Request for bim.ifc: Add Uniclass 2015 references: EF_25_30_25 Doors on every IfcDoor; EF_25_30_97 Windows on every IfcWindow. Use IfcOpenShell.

First a look at what the model holds.

```python
import ifcopenshell

model = ifcopenshell.open("bim.ifc")
print(model.schema)
print("classifications:", [c.Name for c in model.by_type("IfcClassification")])
for ifc_class in ("IfcDoor", "IfcRoof", "IfcStair", "IfcWall", "IfcWindow"):
    print(ifc_class, len(model.by_type(ifc_class)))
```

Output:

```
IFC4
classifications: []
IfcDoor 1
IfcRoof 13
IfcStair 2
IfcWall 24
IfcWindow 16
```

```python
import ifcopenshell
import ifcopenshell.api.classification

model = ifcopenshell.open("bim.ifc")

system = ifcopenshell.api.classification.add_classification(model, classification="Uniclass 2015")

codes = {
    "IfcDoor": ("EF_25_30_25", "Doors"),
    "IfcWindow": ("EF_25_30_97", "Windows"),
}
for ifc_class, (code, name) in codes.items():
    products = model.by_type(ifc_class)
    ifcopenshell.api.classification.add_reference(
        model, products=products, classification=system, identification=code, name=name
    )
    print(code, len(products))

model.write("bim_edited.ifc")
```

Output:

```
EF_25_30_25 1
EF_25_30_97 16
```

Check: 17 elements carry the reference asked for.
